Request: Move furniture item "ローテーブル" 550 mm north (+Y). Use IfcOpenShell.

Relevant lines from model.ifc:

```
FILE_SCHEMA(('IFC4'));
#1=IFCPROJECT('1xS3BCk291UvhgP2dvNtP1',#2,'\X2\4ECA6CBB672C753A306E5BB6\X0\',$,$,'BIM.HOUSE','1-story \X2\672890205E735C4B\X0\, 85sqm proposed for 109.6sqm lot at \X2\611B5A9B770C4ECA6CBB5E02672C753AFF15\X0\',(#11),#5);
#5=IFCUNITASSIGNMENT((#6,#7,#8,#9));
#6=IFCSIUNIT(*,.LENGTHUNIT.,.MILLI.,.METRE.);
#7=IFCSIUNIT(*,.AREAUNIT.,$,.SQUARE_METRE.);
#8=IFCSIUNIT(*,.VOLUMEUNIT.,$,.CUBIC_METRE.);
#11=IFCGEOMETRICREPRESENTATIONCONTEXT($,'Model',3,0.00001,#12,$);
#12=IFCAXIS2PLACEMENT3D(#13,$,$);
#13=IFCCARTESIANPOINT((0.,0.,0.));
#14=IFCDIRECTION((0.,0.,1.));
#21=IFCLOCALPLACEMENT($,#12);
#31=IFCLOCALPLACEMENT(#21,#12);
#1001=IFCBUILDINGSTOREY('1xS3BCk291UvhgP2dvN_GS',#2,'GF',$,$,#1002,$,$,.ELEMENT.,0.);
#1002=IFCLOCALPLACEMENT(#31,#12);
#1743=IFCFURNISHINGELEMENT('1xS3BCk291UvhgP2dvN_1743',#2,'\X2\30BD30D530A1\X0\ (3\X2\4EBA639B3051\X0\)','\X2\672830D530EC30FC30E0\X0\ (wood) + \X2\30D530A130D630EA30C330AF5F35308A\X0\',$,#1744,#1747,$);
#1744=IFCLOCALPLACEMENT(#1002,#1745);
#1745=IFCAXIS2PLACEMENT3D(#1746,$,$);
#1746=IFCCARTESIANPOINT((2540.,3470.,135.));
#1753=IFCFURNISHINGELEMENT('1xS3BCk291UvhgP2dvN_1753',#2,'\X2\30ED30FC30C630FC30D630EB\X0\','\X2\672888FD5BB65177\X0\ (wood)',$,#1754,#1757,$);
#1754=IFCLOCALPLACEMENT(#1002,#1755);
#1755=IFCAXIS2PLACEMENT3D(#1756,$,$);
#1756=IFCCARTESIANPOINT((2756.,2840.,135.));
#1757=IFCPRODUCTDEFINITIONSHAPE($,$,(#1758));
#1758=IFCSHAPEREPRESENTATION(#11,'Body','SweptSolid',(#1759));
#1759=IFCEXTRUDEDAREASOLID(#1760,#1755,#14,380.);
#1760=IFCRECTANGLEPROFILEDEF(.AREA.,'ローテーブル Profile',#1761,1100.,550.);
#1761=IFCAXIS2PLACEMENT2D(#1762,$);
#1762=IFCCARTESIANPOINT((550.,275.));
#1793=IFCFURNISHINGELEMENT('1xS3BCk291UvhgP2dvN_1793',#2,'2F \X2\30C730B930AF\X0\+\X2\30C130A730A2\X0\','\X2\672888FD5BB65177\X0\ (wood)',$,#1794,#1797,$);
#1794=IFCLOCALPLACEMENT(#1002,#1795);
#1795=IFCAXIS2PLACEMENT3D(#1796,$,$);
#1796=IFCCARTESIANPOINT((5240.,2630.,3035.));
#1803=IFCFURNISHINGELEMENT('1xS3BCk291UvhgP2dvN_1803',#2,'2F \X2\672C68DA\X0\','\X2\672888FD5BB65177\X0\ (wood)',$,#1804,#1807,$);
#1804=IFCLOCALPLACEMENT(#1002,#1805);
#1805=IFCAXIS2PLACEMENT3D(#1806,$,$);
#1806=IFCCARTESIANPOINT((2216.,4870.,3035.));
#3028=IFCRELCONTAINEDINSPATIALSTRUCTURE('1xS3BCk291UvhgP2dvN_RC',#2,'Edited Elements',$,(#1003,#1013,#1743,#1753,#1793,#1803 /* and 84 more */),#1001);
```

```python
import ifcopenshell
import ifcopenshell.api.geometry
import ifcopenshell.util.placement
import ifcopenshell.util.unit

model = ifcopenshell.open("model.ifc")
unit_scale = ifcopenshell.util.unit.calculate_unit_scale(model)

item = model.by_guid("1xS3BCk291UvhgP2dvN_1753")
matrix = ifcopenshell.util.placement.get_local_placement(item.ObjectPlacement)
matrix[1, 3] += 0.55 / unit_scale
ifcopenshell.api.geometry.edit_object_placement(model, product=item, matrix=matrix, is_si=False)

print(ifcopenshell.util.placement.get_local_placement(item.ObjectPlacement).round(3) + 0.0)

model.write("model_rev.ifc")
```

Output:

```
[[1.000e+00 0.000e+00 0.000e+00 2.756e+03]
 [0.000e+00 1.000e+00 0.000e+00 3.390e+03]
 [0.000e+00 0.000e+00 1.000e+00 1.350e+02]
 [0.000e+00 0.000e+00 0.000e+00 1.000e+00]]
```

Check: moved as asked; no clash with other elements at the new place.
